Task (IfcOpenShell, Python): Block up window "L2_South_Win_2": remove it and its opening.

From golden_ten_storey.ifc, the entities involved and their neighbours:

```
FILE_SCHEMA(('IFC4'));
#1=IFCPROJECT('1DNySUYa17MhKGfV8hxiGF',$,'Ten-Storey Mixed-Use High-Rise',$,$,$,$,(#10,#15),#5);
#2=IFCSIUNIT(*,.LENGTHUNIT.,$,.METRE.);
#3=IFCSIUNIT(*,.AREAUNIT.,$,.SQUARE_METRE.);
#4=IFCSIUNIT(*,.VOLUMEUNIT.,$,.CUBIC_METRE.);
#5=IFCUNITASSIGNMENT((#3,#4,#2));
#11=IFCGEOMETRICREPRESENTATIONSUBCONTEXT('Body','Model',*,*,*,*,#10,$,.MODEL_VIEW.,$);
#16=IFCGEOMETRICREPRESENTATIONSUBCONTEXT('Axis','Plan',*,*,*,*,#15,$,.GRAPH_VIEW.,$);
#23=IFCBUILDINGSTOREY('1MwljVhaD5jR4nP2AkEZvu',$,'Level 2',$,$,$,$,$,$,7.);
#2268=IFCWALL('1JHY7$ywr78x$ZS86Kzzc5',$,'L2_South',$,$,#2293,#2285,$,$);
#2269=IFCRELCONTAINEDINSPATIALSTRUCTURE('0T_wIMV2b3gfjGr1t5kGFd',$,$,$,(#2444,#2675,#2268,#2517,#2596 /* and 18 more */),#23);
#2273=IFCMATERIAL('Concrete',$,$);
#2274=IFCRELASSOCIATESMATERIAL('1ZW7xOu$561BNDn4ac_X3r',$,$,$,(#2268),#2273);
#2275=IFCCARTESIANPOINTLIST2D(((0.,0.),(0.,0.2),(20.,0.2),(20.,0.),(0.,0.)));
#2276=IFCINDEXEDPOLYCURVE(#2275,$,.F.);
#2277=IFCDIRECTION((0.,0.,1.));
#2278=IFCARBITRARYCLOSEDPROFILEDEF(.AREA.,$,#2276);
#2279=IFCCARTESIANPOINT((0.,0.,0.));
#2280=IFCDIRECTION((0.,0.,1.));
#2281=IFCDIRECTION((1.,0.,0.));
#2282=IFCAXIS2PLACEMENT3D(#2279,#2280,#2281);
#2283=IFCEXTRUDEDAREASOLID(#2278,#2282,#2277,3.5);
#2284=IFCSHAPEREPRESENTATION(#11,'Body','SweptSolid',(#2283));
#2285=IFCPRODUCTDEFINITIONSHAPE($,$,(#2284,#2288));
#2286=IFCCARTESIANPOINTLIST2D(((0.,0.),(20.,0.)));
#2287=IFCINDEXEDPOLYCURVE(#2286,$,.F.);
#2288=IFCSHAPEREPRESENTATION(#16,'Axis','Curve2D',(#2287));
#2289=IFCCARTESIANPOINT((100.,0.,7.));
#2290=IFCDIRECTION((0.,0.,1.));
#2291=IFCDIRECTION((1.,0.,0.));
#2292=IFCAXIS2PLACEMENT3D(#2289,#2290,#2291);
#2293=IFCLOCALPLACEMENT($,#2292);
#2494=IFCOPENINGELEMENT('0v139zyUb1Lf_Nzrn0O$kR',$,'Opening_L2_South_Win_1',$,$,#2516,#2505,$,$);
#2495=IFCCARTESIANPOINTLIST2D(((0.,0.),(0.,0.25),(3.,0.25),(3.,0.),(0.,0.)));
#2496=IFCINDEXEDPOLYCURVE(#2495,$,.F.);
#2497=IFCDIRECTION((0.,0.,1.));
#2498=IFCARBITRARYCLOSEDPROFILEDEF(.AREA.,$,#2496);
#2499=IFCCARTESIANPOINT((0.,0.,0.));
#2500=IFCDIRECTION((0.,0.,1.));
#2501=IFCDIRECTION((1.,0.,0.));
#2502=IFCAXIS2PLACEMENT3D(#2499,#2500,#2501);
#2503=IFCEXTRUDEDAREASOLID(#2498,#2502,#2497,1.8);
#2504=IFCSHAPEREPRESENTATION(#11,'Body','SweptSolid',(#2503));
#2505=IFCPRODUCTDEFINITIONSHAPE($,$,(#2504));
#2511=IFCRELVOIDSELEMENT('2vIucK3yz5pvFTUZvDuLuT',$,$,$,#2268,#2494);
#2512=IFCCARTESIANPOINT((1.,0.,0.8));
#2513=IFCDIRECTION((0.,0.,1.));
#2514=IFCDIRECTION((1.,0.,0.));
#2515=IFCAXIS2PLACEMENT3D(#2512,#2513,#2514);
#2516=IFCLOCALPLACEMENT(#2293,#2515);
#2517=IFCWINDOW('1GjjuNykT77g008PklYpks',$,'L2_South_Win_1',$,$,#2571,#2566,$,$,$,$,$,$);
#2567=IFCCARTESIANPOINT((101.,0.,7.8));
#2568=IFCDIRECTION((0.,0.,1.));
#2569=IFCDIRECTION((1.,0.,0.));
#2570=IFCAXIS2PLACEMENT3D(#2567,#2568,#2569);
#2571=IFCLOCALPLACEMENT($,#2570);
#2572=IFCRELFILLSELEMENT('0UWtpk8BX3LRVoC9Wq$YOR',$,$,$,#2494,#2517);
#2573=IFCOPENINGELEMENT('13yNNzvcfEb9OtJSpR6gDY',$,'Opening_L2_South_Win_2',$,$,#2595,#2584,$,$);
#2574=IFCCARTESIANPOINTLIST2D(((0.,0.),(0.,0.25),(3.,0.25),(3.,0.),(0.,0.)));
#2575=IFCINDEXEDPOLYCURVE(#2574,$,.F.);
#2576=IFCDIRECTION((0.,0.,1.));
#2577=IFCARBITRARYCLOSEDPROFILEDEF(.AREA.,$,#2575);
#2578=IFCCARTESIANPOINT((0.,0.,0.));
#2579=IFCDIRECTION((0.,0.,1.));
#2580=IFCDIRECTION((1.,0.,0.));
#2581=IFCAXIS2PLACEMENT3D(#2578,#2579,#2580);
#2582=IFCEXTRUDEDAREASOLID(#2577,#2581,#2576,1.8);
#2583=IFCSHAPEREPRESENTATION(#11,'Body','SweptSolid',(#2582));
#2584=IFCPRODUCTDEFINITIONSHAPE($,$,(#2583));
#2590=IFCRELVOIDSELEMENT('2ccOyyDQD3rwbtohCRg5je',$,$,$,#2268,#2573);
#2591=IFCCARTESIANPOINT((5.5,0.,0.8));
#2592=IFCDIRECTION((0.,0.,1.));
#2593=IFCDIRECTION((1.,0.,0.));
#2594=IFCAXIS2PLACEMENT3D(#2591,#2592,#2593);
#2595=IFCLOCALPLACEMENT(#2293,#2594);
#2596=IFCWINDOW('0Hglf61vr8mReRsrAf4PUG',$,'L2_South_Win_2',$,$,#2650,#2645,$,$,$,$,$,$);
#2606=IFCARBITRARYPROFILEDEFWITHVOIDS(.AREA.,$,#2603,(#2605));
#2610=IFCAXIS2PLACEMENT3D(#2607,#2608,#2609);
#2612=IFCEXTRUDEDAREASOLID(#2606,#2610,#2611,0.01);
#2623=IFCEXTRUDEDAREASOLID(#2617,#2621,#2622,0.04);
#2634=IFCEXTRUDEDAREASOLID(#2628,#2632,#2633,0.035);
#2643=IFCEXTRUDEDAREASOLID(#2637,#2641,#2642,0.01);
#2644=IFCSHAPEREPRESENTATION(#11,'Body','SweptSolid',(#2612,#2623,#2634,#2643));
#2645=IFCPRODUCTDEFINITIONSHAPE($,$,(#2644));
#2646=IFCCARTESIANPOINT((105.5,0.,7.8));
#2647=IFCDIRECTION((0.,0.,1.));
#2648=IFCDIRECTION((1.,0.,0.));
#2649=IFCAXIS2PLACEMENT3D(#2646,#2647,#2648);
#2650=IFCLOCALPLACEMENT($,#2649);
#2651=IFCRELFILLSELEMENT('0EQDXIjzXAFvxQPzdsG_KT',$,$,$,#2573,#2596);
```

```python
import ifcopenshell
import ifcopenshell.api.feature
import ifcopenshell.api.root
import ifcopenshell.geom
import ifcopenshell.util.shape

model = ifcopenshell.open("golden_ten_storey.ifc")
settings = ifcopenshell.geom.settings()


def volume(element):
    """Net volume in cubic metres, openings subtracted."""
    shape = ifcopenshell.geom.create_shape(settings, element)
    return ifcopenshell.util.shape.get_volume(shape.geometry)


window = model.by_guid("0Hglf61vr8mReRsrAf4PUG")
opening = window.FillsVoids[0].RelatingOpeningElement
wall = opening.VoidsElements[0].RelatingBuildingElement
before = volume(wall)

ifcopenshell.api.root.remove_product(model, product=window)
ifcopenshell.api.feature.remove_feature(model, feature=opening)

after = volume(wall)

print(f"wall volume {before:.3f} -> {after:.3f} m3")

model.write("golden_ten_storey-out.ifc")
```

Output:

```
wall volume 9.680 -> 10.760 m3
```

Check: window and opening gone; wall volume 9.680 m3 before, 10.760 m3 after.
